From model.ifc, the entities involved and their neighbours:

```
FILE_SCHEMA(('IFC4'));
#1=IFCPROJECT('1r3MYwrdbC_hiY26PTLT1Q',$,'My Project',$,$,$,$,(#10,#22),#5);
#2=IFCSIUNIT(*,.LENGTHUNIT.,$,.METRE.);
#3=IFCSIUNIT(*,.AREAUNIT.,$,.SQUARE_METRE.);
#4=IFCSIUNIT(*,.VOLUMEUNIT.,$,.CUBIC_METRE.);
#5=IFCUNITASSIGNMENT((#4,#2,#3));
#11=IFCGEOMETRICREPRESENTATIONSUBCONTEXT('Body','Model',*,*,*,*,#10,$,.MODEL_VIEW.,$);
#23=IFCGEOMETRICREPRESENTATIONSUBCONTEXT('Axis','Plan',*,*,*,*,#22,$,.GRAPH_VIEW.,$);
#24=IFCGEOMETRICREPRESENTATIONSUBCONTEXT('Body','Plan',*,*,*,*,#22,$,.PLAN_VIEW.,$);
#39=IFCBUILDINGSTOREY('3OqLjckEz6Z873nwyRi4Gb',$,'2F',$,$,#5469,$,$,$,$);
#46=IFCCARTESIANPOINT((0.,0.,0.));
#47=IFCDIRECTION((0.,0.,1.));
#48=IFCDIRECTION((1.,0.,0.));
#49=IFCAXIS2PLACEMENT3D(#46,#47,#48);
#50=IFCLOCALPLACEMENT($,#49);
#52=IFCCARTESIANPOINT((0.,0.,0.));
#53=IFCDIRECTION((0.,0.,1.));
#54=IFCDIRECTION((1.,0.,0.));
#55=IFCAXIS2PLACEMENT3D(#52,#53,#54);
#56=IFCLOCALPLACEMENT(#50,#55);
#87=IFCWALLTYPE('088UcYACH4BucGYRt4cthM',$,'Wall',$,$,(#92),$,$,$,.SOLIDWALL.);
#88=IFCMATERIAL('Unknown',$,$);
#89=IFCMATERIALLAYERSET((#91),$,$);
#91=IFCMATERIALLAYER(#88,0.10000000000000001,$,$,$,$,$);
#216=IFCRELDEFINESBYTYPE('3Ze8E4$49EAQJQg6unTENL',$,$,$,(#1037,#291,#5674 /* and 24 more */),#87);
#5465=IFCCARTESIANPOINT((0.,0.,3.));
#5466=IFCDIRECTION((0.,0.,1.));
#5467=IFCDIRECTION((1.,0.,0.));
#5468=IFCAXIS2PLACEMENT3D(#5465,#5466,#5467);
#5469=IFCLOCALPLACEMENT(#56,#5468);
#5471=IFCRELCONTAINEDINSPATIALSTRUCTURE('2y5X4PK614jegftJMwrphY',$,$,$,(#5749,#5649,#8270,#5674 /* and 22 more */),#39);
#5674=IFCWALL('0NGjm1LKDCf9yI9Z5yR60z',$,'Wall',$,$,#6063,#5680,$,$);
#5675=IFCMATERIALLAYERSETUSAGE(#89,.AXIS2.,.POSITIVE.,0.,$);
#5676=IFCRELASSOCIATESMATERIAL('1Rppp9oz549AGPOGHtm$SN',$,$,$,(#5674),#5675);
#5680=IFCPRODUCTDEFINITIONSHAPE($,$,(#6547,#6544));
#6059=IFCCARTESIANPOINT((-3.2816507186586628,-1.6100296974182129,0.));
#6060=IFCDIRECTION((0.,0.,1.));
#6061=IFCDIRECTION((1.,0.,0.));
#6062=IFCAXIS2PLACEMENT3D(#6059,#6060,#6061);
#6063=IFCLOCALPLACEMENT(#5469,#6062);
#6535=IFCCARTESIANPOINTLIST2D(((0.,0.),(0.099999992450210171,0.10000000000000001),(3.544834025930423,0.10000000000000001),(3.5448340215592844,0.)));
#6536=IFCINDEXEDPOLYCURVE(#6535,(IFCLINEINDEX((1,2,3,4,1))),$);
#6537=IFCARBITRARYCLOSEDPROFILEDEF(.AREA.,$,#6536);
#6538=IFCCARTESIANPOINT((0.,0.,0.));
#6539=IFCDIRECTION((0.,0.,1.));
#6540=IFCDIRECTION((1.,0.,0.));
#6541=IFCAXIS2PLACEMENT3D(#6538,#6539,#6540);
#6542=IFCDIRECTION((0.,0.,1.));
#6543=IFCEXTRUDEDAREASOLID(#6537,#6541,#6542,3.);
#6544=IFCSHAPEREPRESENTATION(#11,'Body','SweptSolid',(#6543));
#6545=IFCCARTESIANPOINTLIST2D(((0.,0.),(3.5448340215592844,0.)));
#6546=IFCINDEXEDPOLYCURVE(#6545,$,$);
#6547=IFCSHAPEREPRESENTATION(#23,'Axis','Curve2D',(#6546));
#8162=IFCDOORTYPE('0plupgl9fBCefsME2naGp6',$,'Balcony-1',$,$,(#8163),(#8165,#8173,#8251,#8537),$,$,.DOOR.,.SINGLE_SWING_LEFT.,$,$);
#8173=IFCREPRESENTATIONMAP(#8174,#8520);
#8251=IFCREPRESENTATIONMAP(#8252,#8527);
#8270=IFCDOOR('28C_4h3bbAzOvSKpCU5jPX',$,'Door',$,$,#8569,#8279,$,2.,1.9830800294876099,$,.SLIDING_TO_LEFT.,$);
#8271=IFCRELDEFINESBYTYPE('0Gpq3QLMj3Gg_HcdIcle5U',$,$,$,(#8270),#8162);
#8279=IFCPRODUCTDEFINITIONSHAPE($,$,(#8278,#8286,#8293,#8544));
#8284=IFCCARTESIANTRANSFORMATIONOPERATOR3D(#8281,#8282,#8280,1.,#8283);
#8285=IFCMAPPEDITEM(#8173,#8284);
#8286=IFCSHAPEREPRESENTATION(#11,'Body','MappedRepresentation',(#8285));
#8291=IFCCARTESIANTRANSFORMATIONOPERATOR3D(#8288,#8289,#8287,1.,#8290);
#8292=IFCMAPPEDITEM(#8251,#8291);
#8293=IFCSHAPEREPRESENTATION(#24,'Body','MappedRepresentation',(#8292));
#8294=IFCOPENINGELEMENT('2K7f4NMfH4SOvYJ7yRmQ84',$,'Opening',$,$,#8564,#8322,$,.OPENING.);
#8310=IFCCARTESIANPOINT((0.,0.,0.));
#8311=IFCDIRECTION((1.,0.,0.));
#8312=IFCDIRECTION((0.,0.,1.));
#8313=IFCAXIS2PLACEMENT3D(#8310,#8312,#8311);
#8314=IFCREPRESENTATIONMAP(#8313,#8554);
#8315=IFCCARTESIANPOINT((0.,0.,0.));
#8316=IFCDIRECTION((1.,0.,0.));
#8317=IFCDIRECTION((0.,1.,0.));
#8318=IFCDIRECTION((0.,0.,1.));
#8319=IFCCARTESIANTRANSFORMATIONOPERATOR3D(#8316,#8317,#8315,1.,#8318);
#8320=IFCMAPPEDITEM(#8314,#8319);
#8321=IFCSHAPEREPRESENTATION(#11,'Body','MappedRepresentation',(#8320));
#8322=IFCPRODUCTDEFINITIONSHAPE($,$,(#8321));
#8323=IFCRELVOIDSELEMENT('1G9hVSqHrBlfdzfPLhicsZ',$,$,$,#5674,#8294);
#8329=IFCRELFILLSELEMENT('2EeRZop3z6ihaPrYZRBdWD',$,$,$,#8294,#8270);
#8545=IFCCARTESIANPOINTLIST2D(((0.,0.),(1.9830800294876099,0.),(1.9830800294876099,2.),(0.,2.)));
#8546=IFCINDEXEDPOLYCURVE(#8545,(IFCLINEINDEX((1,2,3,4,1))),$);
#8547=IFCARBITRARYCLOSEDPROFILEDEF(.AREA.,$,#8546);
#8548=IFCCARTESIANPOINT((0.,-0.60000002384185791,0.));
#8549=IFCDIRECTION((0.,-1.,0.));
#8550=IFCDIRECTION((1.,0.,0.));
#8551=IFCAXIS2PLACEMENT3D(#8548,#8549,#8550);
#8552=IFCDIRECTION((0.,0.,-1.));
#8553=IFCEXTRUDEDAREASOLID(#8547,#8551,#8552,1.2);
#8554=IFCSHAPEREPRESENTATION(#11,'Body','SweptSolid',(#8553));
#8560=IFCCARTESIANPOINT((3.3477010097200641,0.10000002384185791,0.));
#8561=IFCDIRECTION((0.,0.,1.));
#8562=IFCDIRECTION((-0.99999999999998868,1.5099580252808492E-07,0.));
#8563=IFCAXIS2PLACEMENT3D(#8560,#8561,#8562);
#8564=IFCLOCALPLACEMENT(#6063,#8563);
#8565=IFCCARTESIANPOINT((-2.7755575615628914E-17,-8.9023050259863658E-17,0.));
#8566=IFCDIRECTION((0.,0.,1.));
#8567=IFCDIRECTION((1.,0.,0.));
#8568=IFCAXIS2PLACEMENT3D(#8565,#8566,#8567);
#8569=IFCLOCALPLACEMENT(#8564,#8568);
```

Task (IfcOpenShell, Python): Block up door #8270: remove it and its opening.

```python
import ifcopenshell
import ifcopenshell.api.feature
import ifcopenshell.api.root
import ifcopenshell.geom
import ifcopenshell.util.shape

model = ifcopenshell.open("model.ifc")
settings = ifcopenshell.geom.settings()


def volume(element):
    """Net volume in cubic metres, openings subtracted."""
    shape = ifcopenshell.geom.create_shape(settings, element)
    return ifcopenshell.util.shape.get_volume(shape.geometry)


door = model.by_guid("28C_4h3bbAzOvSKpCU5jPX")
opening = door.FillsVoids[0].RelatingOpeningElement
wall = opening.VoidsElements[0].RelatingBuildingElement
before = volume(wall)

ifcopenshell.api.root.remove_product(model, product=door)
ifcopenshell.api.feature.remove_feature(model, feature=opening)

after = volume(wall)

print(f"wall volume {before:.3f} -> {after:.3f} m3")

model.write("model_rev.ifc")
```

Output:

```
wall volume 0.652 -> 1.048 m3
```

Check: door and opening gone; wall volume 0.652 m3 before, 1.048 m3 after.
